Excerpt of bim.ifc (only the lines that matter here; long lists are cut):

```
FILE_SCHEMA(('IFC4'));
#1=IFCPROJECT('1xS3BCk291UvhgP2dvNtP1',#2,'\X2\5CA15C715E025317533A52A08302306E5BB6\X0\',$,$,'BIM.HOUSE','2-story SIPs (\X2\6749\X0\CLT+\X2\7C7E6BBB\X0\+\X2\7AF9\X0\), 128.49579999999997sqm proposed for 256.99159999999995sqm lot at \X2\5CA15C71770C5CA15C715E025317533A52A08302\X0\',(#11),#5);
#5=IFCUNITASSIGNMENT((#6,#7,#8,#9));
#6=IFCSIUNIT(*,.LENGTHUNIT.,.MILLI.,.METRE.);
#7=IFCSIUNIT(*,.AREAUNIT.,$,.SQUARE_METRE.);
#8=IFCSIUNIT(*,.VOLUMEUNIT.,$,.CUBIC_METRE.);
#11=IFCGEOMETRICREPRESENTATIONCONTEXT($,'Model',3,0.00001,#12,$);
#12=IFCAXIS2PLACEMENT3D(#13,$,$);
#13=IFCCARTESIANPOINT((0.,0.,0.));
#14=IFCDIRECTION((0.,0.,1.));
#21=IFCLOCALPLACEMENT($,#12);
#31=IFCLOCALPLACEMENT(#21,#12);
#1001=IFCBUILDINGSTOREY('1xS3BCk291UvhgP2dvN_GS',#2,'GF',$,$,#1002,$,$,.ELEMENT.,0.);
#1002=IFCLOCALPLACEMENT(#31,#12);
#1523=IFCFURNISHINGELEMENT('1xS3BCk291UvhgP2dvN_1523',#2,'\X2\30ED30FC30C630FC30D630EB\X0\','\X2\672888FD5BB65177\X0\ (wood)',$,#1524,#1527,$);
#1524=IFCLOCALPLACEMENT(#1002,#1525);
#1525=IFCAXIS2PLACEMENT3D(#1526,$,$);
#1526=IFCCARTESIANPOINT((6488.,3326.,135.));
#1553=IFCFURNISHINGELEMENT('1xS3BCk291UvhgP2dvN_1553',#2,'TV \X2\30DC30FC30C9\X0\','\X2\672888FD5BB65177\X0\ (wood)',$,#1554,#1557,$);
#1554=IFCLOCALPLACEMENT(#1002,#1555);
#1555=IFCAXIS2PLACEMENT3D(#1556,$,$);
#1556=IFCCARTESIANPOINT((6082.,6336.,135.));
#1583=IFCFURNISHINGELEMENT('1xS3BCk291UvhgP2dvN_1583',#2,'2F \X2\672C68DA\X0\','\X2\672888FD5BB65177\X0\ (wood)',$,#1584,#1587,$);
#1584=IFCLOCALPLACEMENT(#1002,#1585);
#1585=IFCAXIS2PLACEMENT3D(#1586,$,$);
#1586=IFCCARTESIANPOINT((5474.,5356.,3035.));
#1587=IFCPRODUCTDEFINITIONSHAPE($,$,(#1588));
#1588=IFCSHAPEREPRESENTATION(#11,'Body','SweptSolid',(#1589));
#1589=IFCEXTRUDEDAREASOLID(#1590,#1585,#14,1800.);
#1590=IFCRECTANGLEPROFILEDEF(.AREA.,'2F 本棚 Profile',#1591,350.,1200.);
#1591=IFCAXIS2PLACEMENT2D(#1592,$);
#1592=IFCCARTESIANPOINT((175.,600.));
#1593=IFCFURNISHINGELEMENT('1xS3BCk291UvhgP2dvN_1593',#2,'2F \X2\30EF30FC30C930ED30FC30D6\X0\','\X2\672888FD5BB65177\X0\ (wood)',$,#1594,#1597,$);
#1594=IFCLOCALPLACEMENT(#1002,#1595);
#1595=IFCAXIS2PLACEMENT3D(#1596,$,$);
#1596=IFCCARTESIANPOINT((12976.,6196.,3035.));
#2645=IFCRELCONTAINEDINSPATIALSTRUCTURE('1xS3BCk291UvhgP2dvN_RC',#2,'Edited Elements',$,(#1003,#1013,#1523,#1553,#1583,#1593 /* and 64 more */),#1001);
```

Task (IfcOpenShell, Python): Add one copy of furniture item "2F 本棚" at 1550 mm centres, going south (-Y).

```python
import numpy as np
import ifcopenshell
import ifcopenshell.api.geometry
import ifcopenshell.api.root
import ifcopenshell.util.element
import ifcopenshell.util.placement

model = ifcopenshell.open("bim.ifc")


def reuse_history(source, copy):
    """copy_class also copies each property set's owner history, people and application; keep the originals."""
    for rel in copy.IsDefinedBy:
        if rel.is_a("IfcRelDefinesByProperties") and (history := rel.RelatingPropertyDefinition.OwnerHistory):
            rel.RelatingPropertyDefinition.OwnerHistory = source.OwnerHistory
            ifcopenshell.util.element.remove_deep2(model, history)


source = model.by_guid("1xS3BCk291UvhgP2dvN_1583")
base = ifcopenshell.util.placement.get_local_placement(source.ObjectPlacement)
step = np.array([0.0, -1.0, 0.0]) * 1550.0

for i in range(1, 2):
    copy = ifcopenshell.api.root.copy_class(model, product=source)
    copy.Representation = ifcopenshell.util.element.copy_deep(
        model, source.Representation, exclude=["IfcGeometricRepresentationContext", "IfcRepresentationMap"]
    )
    reuse_history(source, copy)
    matrix = base.copy()
    matrix[:3, 3] += i * step
    print("added at", matrix[:3, 3].round(3) + 0.0)
    ifcopenshell.api.geometry.edit_object_placement(model, product=copy, matrix=matrix, is_si=False)

model.write("bim_rev.ifc")
```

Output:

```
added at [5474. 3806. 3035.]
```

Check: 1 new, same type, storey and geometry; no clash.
